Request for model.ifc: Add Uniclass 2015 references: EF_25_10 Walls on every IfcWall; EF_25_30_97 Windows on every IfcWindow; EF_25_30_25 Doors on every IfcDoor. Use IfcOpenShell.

First a look at what the model holds.

```python
import ifcopenshell

model = ifcopenshell.open("model.ifc")
print(model.schema)
print("classifications:", [c.Name for c in model.by_type("IfcClassification")])
for ifc_class in ("IfcDoor", "IfcRoof", "IfcStair", "IfcWall", "IfcWindow"):
    print(ifc_class, len(model.by_type(ifc_class)))
```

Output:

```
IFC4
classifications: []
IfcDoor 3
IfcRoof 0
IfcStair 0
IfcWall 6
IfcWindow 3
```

```python
import ifcopenshell
import ifcopenshell.api.classification

model = ifcopenshell.open("model.ifc")

system = ifcopenshell.api.classification.add_classification(model, classification="Uniclass 2015")

codes = {
    "IfcWall": ("EF_25_10", "Walls"),
    "IfcWindow": ("EF_25_30_97", "Windows"),
    "IfcDoor": ("EF_25_30_25", "Doors"),
}
for ifc_class, (code, name) in codes.items():
    products = model.by_type(ifc_class)
    ifcopenshell.api.classification.add_reference(
        model, products=products, classification=system, identification=code, name=name
    )
    print(code, len(products))

model.write("model_rev.ifc")
```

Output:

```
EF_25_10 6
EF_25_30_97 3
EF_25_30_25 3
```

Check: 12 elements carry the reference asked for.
